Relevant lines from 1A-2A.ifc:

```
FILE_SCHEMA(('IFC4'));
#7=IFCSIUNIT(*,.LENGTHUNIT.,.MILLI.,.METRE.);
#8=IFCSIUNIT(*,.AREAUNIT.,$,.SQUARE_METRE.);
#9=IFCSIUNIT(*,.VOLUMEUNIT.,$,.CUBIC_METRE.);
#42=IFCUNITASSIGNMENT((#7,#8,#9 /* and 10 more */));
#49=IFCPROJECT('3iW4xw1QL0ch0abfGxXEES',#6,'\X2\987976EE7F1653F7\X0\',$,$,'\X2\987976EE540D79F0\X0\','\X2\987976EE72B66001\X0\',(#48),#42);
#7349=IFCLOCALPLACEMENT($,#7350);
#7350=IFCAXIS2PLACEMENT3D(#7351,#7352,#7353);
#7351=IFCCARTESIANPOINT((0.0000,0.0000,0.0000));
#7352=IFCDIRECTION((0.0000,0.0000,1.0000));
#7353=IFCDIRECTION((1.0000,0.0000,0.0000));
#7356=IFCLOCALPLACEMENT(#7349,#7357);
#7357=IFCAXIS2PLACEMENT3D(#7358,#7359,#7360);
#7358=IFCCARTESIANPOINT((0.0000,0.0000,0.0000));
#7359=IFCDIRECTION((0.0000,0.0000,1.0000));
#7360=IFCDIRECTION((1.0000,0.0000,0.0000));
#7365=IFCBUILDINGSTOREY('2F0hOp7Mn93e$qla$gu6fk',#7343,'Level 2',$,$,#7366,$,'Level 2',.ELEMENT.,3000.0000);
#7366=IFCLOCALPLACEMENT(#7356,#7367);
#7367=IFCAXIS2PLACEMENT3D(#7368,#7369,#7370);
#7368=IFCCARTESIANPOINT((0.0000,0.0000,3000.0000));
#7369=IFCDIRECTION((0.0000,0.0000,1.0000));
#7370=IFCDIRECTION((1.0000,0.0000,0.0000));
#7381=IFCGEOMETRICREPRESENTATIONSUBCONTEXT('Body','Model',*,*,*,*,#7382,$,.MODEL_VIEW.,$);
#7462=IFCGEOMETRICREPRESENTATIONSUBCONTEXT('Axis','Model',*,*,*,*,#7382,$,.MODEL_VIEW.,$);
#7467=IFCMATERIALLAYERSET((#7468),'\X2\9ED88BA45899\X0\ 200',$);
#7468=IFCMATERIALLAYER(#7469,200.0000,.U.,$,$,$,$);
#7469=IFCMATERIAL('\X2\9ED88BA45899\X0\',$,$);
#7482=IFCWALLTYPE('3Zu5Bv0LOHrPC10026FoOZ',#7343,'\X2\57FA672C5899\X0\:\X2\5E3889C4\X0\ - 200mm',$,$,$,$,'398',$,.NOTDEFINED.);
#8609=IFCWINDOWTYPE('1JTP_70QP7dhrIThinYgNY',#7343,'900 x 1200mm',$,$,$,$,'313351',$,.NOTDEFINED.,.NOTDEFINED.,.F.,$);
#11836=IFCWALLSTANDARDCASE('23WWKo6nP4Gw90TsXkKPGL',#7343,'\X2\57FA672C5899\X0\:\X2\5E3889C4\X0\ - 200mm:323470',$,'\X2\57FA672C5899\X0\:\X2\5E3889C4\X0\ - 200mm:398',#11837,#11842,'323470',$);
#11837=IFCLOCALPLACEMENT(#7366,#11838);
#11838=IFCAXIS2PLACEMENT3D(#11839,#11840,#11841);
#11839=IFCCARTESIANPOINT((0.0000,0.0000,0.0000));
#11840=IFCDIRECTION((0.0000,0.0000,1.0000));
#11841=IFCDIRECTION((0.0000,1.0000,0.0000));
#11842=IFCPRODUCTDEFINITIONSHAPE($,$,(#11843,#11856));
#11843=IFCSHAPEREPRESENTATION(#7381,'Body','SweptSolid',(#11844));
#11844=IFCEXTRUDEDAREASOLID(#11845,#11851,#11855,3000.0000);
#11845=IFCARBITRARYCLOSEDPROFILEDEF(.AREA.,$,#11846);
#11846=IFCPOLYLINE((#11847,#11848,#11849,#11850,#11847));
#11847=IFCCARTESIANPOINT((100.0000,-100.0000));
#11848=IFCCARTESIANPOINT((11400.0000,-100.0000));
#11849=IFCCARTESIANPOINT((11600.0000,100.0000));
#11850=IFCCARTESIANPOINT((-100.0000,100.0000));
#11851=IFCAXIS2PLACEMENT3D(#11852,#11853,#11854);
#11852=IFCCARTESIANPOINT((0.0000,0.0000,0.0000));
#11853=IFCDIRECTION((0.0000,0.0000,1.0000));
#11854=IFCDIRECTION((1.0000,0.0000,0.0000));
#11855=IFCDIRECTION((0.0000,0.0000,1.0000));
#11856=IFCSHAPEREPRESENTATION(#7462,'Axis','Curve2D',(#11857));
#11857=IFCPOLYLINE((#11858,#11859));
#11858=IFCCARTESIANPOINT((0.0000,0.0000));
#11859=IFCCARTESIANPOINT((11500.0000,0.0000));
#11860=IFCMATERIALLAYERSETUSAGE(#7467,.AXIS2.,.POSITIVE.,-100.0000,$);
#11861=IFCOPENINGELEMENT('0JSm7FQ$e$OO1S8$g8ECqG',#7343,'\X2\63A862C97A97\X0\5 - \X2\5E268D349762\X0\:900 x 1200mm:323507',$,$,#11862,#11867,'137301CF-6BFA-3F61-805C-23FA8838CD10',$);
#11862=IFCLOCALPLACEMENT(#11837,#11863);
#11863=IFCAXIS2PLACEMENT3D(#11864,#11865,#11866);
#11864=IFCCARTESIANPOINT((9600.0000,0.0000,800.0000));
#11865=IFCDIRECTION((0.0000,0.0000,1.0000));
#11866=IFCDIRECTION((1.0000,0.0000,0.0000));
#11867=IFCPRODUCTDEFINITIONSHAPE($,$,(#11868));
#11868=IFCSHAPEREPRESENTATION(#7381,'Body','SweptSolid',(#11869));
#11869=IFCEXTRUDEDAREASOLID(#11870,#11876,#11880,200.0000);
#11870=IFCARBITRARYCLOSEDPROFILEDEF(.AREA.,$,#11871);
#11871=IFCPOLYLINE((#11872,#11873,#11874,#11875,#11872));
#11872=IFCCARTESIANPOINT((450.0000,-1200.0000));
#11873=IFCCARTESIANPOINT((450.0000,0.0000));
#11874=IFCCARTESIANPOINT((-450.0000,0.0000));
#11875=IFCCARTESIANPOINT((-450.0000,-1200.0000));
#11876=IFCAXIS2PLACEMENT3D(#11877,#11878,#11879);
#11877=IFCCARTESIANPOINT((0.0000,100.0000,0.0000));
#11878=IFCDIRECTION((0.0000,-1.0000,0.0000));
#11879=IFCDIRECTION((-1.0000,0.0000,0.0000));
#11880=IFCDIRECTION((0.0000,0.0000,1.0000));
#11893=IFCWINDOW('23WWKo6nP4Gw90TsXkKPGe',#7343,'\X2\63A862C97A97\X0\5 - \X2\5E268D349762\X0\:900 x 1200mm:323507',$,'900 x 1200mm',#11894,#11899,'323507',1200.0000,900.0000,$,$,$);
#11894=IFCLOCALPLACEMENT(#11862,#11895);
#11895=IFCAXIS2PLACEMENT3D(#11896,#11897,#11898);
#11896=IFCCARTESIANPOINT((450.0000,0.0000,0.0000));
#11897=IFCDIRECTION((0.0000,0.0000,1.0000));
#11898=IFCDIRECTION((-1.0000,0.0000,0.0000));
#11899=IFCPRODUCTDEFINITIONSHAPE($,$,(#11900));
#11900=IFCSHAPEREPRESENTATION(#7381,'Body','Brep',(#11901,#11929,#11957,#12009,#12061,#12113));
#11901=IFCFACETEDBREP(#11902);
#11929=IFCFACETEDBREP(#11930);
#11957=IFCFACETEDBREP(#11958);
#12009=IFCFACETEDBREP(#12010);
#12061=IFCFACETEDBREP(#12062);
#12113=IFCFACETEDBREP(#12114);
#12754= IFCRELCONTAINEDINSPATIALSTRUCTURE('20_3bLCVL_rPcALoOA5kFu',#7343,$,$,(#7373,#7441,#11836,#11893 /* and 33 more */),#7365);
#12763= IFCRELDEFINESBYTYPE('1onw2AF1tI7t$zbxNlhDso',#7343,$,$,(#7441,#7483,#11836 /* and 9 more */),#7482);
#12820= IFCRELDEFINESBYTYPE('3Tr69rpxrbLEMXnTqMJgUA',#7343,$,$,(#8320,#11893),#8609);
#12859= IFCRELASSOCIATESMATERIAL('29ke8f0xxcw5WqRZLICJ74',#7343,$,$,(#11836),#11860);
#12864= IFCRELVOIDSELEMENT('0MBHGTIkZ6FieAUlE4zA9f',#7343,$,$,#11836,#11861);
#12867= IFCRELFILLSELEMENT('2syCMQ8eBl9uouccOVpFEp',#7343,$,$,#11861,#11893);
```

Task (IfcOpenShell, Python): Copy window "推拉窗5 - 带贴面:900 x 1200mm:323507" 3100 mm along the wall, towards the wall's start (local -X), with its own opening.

```python
import ifcopenshell
import ifcopenshell.api.feature
import ifcopenshell.api.geometry
import ifcopenshell.api.root
import ifcopenshell.geom
import ifcopenshell.util.element
import ifcopenshell.util.placement
import ifcopenshell.util.shape
import ifcopenshell.util.unit

model = ifcopenshell.open("1A-2A.ifc")
unit_scale = ifcopenshell.util.unit.calculate_unit_scale(model)
settings = ifcopenshell.geom.settings()


def volume(element):
    """Net volume in cubic metres, openings subtracted."""
    shape = ifcopenshell.geom.create_shape(settings, element)
    return ifcopenshell.util.shape.get_volume(shape.geometry)


def reuse_history(source, copy):
    """copy_class also copies each property set's owner history, people and application; keep the originals."""
    for rel in copy.IsDefinedBy:
        if rel.is_a("IfcRelDefinesByProperties") and (history := rel.RelatingPropertyDefinition.OwnerHistory):
            rel.RelatingPropertyDefinition.OwnerHistory = source.OwnerHistory
            ifcopenshell.util.element.remove_deep2(model, history)


window = model.by_id(11893)
opening = window.FillsVoids[0].RelatingOpeningElement
wall = opening.VoidsElements[0].RelatingBuildingElement
before = volume(wall)
shift = ifcopenshell.util.placement.get_local_placement(wall.ObjectPlacement)[:3, 0] * -3.1 / unit_scale

# copy_class copies the void relationship, type, container and properties, but no geometry.
new_opening = ifcopenshell.api.root.copy_class(model, product=opening)
new_opening.Representation = ifcopenshell.util.element.copy_deep(
    model, opening.Representation, exclude=["IfcGeometricRepresentationContext", "IfcRepresentationMap"]
)
new_opening.Name = "推拉窗5 - 带贴面:900 x 1200mm"
new_opening.Tag = None
new_window = ifcopenshell.api.root.copy_class(model, product=window)
new_window.Representation = ifcopenshell.util.element.copy_deep(
    model, window.Representation, exclude=["IfcGeometricRepresentationContext", "IfcRepresentationMap"]
)
new_window.Name = "推拉窗5 - 带贴面:900 x 1200mm"
new_window.Tag = None
reuse_history(window, new_window)
ifcopenshell.api.feature.add_filling(model, opening=new_opening, element=new_window)

for old, new in ((opening, new_opening), (window, new_window)):
    matrix = ifcopenshell.util.placement.get_local_placement(old.ObjectPlacement)
    matrix[:3, 3] += shift
    ifcopenshell.api.geometry.edit_object_placement(model, product=new, matrix=matrix, is_si=False)

after = volume(wall)

print(f"wall volume {before:.3f} -> {after:.3f} m3")

model.write("1A-2A_edited.ifc")
```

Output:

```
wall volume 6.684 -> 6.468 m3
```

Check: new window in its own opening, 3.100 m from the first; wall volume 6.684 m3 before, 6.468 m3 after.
